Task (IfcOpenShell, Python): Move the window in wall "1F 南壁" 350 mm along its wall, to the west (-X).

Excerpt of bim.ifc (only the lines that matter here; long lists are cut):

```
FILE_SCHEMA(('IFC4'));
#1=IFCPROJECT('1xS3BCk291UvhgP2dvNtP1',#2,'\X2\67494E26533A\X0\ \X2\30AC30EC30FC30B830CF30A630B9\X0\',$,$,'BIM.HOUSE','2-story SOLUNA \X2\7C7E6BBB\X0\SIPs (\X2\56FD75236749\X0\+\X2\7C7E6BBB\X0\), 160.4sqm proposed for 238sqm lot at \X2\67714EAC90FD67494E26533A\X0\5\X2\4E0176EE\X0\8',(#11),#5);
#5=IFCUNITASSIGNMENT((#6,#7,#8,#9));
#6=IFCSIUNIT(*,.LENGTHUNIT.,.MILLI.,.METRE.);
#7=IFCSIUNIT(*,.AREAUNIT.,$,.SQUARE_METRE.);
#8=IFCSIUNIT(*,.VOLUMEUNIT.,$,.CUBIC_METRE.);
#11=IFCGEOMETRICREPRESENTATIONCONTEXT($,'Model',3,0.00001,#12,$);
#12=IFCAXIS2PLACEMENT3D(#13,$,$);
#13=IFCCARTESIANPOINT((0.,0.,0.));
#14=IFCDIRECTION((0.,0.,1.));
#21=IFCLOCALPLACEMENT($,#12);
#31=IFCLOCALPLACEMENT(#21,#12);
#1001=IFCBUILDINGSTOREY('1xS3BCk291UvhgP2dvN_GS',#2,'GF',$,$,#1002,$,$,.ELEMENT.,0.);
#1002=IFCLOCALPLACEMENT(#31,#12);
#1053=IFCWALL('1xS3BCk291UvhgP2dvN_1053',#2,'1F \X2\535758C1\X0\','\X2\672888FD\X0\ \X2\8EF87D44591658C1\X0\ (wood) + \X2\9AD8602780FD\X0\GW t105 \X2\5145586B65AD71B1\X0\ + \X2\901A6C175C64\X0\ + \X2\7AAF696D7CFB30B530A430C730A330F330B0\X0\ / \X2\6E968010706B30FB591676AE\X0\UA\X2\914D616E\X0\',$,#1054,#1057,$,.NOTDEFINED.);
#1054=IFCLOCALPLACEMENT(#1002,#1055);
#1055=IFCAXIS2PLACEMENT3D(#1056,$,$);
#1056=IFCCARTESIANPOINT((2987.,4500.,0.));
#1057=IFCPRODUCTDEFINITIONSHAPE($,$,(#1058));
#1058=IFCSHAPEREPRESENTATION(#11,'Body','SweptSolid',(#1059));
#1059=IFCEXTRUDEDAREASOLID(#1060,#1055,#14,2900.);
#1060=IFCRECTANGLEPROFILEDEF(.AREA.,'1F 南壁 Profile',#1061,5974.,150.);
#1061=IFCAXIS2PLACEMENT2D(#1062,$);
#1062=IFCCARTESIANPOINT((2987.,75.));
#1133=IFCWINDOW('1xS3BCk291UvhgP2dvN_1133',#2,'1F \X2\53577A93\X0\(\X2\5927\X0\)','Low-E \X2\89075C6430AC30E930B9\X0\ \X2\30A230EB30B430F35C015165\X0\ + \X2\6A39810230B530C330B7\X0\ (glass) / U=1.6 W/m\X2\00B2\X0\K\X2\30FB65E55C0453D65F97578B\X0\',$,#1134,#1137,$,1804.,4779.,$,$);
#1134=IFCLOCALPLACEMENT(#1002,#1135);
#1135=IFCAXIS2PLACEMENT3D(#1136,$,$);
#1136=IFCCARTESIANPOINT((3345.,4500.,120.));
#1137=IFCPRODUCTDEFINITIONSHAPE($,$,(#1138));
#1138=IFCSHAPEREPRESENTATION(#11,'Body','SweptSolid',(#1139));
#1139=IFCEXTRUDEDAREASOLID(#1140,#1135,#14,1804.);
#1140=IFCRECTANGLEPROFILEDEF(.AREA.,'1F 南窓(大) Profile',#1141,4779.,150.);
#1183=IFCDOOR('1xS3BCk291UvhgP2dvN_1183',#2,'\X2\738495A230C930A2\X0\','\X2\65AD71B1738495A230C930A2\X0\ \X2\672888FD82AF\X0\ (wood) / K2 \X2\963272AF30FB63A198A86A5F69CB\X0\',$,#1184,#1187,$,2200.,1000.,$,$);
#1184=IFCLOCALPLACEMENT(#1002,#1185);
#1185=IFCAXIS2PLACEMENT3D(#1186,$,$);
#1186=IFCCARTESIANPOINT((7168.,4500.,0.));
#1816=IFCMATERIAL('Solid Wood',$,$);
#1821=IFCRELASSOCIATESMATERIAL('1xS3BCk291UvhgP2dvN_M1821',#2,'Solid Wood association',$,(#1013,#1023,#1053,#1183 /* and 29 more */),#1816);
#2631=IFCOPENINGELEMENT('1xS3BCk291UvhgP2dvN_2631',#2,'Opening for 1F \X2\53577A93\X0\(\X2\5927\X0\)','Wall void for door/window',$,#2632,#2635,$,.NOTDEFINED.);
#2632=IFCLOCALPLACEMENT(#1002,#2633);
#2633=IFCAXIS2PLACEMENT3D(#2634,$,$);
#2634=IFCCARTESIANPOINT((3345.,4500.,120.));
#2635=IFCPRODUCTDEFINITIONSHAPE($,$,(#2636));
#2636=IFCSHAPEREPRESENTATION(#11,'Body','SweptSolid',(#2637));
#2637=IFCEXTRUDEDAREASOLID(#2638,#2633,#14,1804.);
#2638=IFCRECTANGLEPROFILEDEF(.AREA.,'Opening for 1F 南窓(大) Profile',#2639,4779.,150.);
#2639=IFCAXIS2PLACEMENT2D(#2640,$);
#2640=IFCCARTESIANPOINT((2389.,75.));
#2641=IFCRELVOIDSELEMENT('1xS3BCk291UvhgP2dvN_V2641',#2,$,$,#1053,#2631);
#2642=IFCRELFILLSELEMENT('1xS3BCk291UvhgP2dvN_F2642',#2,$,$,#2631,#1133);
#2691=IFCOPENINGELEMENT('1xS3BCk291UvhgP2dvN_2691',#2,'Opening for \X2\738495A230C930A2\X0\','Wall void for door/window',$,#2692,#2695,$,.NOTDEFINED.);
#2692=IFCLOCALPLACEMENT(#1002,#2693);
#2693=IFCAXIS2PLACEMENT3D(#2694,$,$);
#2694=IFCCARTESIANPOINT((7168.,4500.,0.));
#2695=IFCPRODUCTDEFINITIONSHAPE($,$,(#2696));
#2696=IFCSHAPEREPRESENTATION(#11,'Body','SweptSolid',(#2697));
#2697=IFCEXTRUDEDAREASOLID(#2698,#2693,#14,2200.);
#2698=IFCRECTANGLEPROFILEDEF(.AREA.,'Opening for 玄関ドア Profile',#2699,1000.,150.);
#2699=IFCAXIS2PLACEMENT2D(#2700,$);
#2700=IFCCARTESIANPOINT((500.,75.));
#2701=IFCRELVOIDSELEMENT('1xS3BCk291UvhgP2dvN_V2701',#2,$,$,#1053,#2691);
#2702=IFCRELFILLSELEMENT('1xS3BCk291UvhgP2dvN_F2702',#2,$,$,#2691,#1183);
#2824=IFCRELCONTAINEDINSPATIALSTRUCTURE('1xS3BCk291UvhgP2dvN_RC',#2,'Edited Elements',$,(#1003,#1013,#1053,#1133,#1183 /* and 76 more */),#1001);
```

```python
import ifcopenshell
import ifcopenshell.api.geometry
import ifcopenshell.util.placement
import ifcopenshell.util.unit

model = ifcopenshell.open("bim.ifc")
unit_scale = ifcopenshell.util.unit.calculate_unit_scale(model)

window = model.by_guid("1xS3BCk291UvhgP2dvN_1133")
opening = window.FillsVoids[0].RelatingOpeningElement
wall = opening.VoidsElements[0].RelatingBuildingElement

wall_matrix = ifcopenshell.util.placement.get_local_placement(wall.ObjectPlacement)
shift = wall_matrix[:3, 0] * -0.35 / unit_scale
before = ifcopenshell.util.placement.get_local_placement(window.ObjectPlacement)[:3, 3].copy()

# The window is not placed relative to its opening, so move both.
for product in (opening, window):
    matrix = ifcopenshell.util.placement.get_local_placement(product.ObjectPlacement)
    matrix[:3, 3] += shift
    ifcopenshell.api.geometry.edit_object_placement(model, product=product, matrix=matrix, is_si=False)

after = ifcopenshell.util.placement.get_local_placement(window.ObjectPlacement)[:3, 3]
print("window moved by", (after - before).round(3) + 0.0)

model.write("bim_v2.ifc")
```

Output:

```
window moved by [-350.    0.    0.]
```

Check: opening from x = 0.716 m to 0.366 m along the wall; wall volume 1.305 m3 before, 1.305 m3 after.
